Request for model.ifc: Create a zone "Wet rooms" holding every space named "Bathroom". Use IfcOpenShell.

First a look at what the model holds.

```python
import ifcopenshell

model = ifcopenshell.open("model.ifc")
print(model.schema)
seen = {}
for space in model.by_type("IfcSpace"):
    seen[space.LongName] = seen.get(space.LongName, 0) + 1
for name, count in sorted(seen.items(), key=str):
    print(count, "x", name)
print("zones:", [z.Name for z in model.by_type("IfcZone")][:20])
```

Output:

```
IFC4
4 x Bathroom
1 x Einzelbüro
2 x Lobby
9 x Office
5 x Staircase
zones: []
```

```python
import ifcopenshell
import ifcopenshell.api.group
import ifcopenshell.api.root

model = ifcopenshell.open("model.ifc")

names = {"Bathroom"}
spaces = [s for s in model.by_type("IfcSpace") if s.LongName in names]

zone = ifcopenshell.api.root.create_entity(model, ifc_class="IfcZone", name="Wet rooms")
ifcopenshell.api.group.assign_group(model, products=spaces, group=zone)
print(len(spaces), "spaces in", zone.Name)

model.write("model_edited.ifc")
```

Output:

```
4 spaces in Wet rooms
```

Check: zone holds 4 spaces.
